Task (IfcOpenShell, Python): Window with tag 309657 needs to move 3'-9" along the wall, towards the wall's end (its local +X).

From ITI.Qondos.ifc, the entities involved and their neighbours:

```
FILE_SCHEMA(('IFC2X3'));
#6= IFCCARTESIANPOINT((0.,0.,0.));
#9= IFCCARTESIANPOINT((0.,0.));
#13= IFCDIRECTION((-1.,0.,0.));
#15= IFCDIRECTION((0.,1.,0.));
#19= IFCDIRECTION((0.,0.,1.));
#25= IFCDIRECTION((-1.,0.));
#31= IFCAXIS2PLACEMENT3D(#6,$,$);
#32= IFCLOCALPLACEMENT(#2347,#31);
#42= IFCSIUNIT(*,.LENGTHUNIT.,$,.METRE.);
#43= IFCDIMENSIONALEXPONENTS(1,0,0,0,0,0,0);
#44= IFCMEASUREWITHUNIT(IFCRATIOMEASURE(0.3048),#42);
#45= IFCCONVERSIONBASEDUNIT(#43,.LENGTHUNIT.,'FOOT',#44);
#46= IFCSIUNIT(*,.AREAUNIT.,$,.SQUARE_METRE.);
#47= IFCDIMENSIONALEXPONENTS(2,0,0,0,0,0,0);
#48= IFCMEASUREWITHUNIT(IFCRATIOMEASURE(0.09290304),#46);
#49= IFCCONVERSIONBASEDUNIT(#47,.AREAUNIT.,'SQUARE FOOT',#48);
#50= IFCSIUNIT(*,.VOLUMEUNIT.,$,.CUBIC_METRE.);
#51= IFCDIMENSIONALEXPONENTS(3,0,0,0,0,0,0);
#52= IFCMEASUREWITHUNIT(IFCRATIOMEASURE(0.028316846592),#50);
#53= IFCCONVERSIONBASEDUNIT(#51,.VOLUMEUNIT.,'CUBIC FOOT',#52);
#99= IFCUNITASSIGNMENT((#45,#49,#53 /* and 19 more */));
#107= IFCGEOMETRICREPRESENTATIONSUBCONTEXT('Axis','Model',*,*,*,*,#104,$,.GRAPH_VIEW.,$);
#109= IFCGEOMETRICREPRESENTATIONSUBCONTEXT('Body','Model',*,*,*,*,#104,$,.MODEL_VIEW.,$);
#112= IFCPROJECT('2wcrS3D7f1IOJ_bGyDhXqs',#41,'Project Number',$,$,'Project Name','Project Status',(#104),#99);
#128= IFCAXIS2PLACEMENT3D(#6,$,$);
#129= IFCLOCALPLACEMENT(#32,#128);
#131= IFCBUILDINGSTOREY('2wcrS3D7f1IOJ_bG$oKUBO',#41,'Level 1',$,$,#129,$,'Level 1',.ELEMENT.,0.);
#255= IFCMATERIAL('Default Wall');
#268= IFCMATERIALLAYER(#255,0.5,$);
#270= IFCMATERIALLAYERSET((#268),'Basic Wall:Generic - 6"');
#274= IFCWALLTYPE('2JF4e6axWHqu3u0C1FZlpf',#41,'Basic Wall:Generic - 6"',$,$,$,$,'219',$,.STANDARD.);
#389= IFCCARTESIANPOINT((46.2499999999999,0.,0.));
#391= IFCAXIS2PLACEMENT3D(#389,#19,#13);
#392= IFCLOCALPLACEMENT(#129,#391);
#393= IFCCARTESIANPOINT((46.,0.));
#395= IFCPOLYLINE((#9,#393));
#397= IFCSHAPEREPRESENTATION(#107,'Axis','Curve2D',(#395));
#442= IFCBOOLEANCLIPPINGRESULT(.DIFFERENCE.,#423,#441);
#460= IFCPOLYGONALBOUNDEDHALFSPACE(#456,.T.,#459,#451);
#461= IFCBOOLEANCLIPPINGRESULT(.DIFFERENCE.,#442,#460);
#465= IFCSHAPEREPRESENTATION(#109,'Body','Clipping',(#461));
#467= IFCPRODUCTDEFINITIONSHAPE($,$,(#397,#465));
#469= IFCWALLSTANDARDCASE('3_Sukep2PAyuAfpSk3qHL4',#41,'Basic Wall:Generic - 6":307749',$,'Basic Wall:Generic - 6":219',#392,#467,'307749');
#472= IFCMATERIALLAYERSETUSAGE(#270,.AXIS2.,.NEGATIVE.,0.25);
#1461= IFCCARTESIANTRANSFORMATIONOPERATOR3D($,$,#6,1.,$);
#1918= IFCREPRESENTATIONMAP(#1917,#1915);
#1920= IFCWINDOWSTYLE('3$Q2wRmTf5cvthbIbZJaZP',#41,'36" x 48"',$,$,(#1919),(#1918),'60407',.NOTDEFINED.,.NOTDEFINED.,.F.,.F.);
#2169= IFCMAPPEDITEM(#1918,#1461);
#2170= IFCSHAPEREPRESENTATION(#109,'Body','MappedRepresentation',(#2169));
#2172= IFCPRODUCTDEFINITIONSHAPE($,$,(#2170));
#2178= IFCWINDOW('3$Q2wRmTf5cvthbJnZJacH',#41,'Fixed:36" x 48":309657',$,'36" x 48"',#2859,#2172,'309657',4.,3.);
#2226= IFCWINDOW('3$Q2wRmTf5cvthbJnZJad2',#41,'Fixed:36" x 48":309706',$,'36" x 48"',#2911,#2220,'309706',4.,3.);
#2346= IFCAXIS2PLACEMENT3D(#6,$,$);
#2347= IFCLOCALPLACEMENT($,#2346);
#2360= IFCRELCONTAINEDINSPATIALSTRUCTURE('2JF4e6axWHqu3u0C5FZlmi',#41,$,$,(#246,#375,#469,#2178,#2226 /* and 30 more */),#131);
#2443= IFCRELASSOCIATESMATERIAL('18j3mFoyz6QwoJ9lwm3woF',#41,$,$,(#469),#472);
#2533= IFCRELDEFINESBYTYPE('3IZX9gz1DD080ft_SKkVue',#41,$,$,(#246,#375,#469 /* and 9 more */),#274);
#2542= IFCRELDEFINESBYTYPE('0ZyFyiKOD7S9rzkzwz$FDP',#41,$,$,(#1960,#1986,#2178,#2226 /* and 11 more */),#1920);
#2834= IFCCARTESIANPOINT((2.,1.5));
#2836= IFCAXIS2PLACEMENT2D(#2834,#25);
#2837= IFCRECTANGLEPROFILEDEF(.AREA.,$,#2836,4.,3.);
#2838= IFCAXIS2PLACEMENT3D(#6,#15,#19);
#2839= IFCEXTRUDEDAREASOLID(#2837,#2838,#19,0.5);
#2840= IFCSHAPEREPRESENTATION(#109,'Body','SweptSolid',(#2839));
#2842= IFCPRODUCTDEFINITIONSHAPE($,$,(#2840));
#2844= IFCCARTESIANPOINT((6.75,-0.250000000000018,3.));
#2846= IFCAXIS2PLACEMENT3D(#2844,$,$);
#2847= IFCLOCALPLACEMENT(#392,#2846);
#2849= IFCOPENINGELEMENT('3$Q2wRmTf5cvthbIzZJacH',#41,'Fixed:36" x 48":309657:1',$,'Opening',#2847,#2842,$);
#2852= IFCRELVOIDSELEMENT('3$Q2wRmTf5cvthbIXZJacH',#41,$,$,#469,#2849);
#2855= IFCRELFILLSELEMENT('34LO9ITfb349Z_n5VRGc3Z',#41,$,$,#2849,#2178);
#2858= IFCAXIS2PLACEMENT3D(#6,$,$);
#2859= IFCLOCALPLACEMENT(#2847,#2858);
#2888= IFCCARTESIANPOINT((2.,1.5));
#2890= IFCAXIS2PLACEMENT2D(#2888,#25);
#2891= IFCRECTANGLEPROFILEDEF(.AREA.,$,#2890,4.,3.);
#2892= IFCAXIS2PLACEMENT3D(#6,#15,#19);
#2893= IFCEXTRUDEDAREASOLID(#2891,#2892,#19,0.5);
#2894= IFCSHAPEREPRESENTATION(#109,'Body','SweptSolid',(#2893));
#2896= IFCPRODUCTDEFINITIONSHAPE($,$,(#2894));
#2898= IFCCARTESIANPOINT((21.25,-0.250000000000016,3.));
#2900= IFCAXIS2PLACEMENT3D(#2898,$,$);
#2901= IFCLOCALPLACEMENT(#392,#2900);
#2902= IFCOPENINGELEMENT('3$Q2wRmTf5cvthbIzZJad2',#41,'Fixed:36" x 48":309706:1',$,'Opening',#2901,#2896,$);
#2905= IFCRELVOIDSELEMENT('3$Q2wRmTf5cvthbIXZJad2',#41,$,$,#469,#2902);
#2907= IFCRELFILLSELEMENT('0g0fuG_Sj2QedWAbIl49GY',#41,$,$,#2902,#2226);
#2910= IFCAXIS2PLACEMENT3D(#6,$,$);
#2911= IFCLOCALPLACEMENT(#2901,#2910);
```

```python
import ifcopenshell
import ifcopenshell.api.geometry
import ifcopenshell.util.placement
import ifcopenshell.util.unit

model = ifcopenshell.open("ITI.Qondos.ifc")
unit_scale = ifcopenshell.util.unit.calculate_unit_scale(model)

window = model.by_guid("3$Q2wRmTf5cvthbJnZJacH")
opening = window.FillsVoids[0].RelatingOpeningElement
wall = opening.VoidsElements[0].RelatingBuildingElement

wall_matrix = ifcopenshell.util.placement.get_local_placement(wall.ObjectPlacement)
shift = wall_matrix[:3, 0] * 45 * 0.0254 / unit_scale
before = ifcopenshell.util.placement.get_local_placement(window.ObjectPlacement)[:3, 3].copy()

# The window is placed relative to its opening, so it follows when the opening moves.
matrix = ifcopenshell.util.placement.get_local_placement(opening.ObjectPlacement)
matrix[:3, 3] += shift
ifcopenshell.api.geometry.edit_object_placement(
    model, product=opening, matrix=matrix, is_si=False, should_transform_children=True
)

after = ifcopenshell.util.placement.get_local_placement(window.ObjectPlacement)[:3, 3]
print("window moved by", (after - before).round(3) + 0.0)

model.write("ITI.Qondos_updated.ifc")
```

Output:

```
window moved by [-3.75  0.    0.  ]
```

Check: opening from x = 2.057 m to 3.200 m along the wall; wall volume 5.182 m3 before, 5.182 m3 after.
